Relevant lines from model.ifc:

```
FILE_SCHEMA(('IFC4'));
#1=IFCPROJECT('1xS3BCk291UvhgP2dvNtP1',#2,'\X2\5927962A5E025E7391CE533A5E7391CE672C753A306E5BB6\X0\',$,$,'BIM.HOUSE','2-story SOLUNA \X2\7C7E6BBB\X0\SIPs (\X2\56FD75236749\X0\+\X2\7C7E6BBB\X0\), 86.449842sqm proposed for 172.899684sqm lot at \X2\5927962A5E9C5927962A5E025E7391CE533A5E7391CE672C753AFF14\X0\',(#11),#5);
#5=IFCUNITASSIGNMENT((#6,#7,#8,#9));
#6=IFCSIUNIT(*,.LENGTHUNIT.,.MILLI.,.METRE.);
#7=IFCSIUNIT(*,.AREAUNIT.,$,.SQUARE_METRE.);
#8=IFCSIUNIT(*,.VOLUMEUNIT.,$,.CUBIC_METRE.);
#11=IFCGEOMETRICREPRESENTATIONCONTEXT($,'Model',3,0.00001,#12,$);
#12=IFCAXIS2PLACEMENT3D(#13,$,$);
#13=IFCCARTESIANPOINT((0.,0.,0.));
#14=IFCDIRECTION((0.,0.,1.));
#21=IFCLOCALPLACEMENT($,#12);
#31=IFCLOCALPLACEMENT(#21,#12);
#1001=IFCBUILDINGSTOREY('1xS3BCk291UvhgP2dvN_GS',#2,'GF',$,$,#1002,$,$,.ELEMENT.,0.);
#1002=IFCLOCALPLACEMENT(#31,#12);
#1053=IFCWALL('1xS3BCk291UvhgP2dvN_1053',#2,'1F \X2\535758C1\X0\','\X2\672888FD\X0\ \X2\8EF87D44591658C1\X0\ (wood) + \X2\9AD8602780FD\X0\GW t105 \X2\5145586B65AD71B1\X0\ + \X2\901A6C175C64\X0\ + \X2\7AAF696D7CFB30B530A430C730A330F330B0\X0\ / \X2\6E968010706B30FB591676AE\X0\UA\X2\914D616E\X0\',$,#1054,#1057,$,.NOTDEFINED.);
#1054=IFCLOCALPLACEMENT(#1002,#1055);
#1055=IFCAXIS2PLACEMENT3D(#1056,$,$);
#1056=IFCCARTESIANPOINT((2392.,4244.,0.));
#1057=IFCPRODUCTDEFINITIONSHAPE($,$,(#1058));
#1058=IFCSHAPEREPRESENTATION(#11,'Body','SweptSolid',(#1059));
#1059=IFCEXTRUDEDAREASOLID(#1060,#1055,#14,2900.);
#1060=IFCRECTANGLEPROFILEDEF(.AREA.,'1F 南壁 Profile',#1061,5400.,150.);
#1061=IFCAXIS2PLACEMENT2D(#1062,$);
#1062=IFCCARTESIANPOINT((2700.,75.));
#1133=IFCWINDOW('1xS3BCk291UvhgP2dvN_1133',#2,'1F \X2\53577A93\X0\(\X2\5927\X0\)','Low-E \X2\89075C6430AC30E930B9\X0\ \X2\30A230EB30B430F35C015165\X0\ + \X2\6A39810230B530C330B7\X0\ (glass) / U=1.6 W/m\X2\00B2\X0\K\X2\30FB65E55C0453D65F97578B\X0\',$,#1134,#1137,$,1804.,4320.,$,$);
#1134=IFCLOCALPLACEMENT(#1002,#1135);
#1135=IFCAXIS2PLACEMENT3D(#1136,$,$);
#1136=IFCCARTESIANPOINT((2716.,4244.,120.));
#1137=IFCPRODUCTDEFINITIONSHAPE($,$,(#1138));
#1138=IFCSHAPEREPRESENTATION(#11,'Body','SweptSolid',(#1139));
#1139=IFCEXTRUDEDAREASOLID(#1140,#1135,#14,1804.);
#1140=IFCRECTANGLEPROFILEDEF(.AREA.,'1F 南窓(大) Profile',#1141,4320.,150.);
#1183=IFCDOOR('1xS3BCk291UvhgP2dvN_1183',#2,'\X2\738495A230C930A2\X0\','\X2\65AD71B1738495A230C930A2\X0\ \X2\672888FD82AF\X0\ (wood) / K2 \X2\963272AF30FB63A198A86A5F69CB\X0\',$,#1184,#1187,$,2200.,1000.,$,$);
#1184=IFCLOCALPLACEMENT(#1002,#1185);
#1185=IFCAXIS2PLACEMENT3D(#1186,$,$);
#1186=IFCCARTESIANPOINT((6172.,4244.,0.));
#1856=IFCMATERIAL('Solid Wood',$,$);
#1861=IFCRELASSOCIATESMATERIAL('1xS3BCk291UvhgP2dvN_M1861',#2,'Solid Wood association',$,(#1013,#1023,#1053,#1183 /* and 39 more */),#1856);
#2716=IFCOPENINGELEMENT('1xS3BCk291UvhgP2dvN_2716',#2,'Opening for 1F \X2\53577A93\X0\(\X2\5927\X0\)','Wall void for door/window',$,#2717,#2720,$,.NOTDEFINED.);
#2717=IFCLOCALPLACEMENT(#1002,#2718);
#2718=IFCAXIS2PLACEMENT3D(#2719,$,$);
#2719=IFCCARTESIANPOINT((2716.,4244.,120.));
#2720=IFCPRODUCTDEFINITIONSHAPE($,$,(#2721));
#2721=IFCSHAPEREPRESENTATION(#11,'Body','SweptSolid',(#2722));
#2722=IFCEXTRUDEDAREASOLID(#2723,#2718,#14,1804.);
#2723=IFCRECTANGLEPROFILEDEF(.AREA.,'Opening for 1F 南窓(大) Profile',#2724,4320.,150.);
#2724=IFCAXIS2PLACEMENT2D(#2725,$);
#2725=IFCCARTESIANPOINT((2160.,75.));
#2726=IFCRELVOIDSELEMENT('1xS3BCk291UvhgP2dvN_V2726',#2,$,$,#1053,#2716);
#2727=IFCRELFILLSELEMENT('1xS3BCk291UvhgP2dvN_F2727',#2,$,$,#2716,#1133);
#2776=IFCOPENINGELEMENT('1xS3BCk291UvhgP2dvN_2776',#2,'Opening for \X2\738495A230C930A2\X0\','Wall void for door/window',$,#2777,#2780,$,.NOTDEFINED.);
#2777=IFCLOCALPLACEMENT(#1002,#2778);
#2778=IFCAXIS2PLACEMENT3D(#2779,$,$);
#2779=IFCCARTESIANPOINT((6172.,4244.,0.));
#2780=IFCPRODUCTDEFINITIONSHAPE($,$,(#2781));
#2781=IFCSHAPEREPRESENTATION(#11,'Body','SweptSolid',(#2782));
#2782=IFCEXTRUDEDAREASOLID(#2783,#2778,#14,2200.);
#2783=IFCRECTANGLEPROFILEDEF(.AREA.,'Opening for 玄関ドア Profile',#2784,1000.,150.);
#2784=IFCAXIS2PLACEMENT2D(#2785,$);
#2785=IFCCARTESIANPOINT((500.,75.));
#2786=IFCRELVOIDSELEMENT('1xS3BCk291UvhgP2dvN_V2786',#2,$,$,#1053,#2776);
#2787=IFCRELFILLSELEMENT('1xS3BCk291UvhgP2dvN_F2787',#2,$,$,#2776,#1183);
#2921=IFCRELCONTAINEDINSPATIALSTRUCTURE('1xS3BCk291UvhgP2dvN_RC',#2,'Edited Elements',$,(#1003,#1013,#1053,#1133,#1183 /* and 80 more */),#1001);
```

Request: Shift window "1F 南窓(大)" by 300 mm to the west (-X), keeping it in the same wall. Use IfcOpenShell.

```python
import ifcopenshell
import ifcopenshell.api.geometry
import ifcopenshell.util.placement

model = ifcopenshell.open("model.ifc")

window = model.by_guid("1xS3BCk291UvhgP2dvN_1133")
opening = window.FillsVoids[0].RelatingOpeningElement
wall = opening.VoidsElements[0].RelatingBuildingElement

wall_matrix = ifcopenshell.util.placement.get_local_placement(wall.ObjectPlacement)
shift = wall_matrix[:3, 0] * -300.0
before = ifcopenshell.util.placement.get_local_placement(window.ObjectPlacement)[:3, 3].copy()

# The window is not placed relative to its opening, so move both.
for product in (opening, window):
    matrix = ifcopenshell.util.placement.get_local_placement(product.ObjectPlacement)
    matrix[:3, 3] += shift
    ifcopenshell.api.geometry.edit_object_placement(model, product=product, matrix=matrix, is_si=False)

after = ifcopenshell.util.placement.get_local_placement(window.ObjectPlacement)[:3, 3]
print("window moved by", (after - before).round(3) + 0.0)

model.write("model-out.ifc")
```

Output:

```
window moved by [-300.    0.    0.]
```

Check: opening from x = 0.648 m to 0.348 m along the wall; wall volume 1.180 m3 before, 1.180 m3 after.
